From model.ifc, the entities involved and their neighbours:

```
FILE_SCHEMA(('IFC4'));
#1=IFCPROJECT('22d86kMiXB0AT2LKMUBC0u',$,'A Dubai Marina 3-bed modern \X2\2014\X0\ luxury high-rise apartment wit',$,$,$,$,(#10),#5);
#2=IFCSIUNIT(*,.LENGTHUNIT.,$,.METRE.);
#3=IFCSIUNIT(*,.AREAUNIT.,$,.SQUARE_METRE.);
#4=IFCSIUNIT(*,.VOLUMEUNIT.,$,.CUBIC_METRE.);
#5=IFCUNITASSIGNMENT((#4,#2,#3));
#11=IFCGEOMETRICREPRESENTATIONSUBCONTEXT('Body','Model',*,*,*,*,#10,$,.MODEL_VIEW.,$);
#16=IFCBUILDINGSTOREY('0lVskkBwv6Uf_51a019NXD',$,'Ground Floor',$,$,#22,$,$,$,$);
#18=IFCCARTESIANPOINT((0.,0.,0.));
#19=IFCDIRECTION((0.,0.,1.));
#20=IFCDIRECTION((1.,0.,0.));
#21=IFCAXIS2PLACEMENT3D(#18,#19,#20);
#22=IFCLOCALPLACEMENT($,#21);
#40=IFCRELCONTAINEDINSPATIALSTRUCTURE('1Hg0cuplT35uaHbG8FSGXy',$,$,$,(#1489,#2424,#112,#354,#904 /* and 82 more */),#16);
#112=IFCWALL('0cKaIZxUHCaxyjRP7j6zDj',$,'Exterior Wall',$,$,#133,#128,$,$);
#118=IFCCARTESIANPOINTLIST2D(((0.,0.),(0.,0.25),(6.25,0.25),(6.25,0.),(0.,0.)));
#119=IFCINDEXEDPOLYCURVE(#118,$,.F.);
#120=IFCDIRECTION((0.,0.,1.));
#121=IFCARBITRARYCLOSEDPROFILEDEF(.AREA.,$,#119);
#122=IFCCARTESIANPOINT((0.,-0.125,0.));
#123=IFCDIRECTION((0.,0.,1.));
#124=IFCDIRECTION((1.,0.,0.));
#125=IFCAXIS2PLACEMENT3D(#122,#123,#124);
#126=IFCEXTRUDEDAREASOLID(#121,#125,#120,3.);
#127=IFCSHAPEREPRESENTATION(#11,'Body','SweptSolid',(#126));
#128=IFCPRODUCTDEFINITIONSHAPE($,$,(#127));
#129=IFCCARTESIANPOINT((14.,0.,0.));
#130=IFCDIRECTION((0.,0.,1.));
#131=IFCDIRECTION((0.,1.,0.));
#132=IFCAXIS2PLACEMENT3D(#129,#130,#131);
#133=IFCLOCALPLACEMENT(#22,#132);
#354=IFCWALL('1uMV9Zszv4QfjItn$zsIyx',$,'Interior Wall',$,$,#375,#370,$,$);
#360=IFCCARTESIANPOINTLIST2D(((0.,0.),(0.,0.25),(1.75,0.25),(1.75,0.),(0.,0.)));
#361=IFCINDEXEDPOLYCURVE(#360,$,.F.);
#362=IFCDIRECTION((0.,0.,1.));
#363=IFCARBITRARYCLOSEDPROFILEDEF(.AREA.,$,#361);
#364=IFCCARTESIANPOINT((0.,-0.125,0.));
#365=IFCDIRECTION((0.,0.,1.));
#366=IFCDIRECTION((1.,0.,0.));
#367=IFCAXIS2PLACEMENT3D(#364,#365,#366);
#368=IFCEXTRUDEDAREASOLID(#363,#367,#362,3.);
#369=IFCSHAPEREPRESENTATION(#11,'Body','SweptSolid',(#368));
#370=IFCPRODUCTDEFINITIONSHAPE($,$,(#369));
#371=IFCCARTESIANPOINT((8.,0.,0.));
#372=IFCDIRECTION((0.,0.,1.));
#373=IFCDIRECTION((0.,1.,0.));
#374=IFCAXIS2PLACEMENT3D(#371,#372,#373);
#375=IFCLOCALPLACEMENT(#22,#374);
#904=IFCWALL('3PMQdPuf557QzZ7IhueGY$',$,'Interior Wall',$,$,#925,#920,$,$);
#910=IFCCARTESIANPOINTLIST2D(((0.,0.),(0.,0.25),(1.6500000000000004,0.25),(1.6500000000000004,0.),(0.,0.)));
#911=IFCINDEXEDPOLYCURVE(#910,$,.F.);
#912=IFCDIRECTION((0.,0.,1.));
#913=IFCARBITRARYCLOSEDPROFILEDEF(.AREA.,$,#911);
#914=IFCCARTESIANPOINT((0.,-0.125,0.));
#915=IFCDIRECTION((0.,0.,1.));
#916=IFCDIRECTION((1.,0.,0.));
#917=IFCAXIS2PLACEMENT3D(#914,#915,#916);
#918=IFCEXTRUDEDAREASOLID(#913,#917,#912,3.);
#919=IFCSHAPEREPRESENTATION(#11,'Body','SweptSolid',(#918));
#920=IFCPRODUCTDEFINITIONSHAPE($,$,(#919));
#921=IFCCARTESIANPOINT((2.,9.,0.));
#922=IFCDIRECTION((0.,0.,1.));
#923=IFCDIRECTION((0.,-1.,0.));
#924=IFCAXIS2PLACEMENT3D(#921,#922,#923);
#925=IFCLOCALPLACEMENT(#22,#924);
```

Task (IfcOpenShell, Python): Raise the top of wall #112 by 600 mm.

```python
import ifcopenshell
import ifcopenshell.geom
import ifcopenshell.util.representation
import ifcopenshell.util.shape

model = ifcopenshell.open("model.ifc")
settings = ifcopenshell.geom.settings()


def volume(element):
    """Net volume in cubic metres, openings subtracted."""
    shape = ifcopenshell.geom.create_shape(settings, element)
    return ifcopenshell.util.shape.get_volume(shape.geometry)


wall = model.by_guid("0cKaIZxUHCaxyjRP7j6zDj")
before = volume(wall)

body = ifcopenshell.util.representation.get_representation(wall, "Model", "Body")
solid = body.Items[0]
old_height = solid.Depth
solid.Depth += 0.6
after = volume(wall)

print(f"height {old_height:g} -> {solid.Depth:g}, volume {before:.3f} -> {after:.3f} m3")

model.write("model-out.ifc")
```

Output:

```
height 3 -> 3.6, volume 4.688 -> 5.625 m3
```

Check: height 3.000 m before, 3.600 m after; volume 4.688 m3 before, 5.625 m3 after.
